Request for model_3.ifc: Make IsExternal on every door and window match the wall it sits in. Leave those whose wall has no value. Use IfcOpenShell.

First a look at what the model holds.

```python
import ifcopenshell
import ifcopenshell.util.element

model = ifcopenshell.open("model_3.ifc")
print(model.schema)
seen = {}
for e in model.by_type("IfcDoor") + model.by_type("IfcWindow"):
    if not e.FillsVoids:
        continue
    host = e.FillsVoids[0].RelatingOpeningElement.VoidsElements[0].RelatingBuildingElement
    own = ifcopenshell.util.element.get_pset(e, f"Pset_{e.is_a()[3:].removesuffix('StandardCase')}Common", "IsExternal")
    wall = ifcopenshell.util.element.get_pset(host, "Pset_WallCommon", "IsExternal")
    seen[e.is_a(), own, wall] = seen.get((e.is_a(), own, wall), 0) + 1
for (cls, own, wall), count in sorted(seen.items(), key=str):
    print(count, cls, "IsExternal:", own, "| host wall:", wall)
```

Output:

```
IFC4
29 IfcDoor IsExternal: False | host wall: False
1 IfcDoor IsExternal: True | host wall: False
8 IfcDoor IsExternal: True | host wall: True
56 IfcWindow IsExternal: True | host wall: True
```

```python
import ifcopenshell
import ifcopenshell.api.pset
import ifcopenshell.util.element

model = ifcopenshell.open("model_3.ifc")

count = 0
for ifc_class, pset_name in (("IfcDoor", "Pset_DoorCommon"), ("IfcWindow", "Pset_WindowCommon")):
    for e in model.by_type(ifc_class):
        if not e.FillsVoids:
            continue
        host = e.FillsVoids[0].RelatingOpeningElement.VoidsElements[0].RelatingBuildingElement
        external = ifcopenshell.util.element.get_pset(host, "Pset_WallCommon", "IsExternal")
        if external is None or ifcopenshell.util.element.get_pset(e, pset_name, "IsExternal") == external:
            continue
        pset = ifcopenshell.api.pset.add_pset(model, product=e, name=pset_name)
        ifcopenshell.api.pset.edit_pset(model, pset=pset, properties={"IsExternal": external})
        count += 1

print(count, "updated")

model.write("model_3_updated.ifc")
```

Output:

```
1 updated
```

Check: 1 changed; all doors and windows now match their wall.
